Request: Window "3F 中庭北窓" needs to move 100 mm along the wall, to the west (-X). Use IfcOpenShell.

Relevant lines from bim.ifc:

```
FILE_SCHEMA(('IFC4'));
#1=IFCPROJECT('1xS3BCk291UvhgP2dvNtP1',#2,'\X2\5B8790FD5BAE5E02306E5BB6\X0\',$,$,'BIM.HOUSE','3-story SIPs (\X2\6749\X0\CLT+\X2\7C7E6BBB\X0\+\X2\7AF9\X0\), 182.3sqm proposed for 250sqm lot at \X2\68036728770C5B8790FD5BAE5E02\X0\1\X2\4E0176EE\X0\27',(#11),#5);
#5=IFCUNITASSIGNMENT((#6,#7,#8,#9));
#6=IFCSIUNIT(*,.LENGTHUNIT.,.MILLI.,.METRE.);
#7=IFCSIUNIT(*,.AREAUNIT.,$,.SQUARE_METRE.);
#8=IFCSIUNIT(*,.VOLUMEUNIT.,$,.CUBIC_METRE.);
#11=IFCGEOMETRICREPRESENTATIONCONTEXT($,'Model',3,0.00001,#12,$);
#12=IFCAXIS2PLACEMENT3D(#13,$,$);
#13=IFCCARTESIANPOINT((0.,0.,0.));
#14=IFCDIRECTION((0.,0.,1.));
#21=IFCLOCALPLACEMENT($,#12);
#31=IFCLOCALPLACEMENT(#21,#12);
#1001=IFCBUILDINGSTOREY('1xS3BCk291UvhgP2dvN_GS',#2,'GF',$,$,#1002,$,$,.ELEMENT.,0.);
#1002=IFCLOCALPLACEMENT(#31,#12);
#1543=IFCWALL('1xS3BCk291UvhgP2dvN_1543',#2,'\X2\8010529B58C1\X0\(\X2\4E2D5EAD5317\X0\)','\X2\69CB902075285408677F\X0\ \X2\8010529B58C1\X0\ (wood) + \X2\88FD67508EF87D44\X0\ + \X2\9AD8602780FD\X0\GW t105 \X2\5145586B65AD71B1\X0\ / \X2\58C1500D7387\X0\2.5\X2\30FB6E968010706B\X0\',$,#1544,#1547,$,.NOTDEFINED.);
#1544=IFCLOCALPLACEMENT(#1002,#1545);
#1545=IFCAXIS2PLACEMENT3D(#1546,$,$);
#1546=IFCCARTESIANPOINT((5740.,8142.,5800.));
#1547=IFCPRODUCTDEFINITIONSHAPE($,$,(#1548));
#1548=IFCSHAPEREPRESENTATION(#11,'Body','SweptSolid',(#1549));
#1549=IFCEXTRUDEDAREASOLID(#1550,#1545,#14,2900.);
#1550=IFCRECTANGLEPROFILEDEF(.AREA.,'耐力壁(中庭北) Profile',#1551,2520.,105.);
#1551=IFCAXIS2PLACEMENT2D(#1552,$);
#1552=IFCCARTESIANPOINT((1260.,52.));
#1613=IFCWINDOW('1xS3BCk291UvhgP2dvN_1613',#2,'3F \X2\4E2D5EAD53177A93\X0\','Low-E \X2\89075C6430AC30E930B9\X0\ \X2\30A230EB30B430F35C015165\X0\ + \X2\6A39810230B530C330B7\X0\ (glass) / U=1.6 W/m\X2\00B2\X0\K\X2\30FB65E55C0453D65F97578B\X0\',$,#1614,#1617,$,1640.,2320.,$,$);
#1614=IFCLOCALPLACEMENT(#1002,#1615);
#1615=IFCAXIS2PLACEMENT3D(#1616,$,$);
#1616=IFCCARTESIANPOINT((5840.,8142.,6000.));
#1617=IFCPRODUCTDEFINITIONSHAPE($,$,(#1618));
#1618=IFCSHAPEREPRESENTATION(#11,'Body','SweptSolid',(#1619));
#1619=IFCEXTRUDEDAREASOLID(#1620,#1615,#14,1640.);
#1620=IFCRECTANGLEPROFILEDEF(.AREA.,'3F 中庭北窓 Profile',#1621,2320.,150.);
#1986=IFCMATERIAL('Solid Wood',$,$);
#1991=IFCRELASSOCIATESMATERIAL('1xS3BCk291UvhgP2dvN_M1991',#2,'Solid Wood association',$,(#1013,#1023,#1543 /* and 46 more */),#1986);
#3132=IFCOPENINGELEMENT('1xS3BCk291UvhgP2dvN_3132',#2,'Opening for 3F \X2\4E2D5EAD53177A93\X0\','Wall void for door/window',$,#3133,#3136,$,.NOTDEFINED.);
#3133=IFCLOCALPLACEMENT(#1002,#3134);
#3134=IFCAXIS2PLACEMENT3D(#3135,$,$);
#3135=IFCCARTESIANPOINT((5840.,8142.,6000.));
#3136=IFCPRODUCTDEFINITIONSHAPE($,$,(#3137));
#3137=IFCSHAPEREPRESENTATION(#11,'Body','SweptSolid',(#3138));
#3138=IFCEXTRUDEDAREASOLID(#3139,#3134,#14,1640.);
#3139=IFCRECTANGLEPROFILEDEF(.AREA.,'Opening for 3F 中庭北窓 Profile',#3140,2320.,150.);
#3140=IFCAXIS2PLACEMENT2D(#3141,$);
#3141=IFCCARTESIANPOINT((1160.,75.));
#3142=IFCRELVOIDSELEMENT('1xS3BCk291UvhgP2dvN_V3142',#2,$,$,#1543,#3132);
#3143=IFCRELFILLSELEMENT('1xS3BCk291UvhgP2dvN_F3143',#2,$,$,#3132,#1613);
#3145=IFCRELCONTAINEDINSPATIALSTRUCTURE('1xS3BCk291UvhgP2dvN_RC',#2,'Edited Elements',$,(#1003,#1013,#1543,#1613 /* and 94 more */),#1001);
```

```python
import ifcopenshell
import ifcopenshell.api.geometry
import ifcopenshell.util.placement

model = ifcopenshell.open("bim.ifc")

window = model.by_id(1613)
opening = window.FillsVoids[0].RelatingOpeningElement
wall = opening.VoidsElements[0].RelatingBuildingElement

wall_matrix = ifcopenshell.util.placement.get_local_placement(wall.ObjectPlacement)
shift = wall_matrix[:3, 0] * -100.0
before = ifcopenshell.util.placement.get_local_placement(window.ObjectPlacement)[:3, 3].copy()

# The window is not placed relative to its opening, so move both.
for product in (opening, window):
    matrix = ifcopenshell.util.placement.get_local_placement(product.ObjectPlacement)
    matrix[:3, 3] += shift
    ifcopenshell.api.geometry.edit_object_placement(model, product=product, matrix=matrix, is_si=False)

after = ifcopenshell.util.placement.get_local_placement(window.ObjectPlacement)[:3, 3]
print("window moved by", (after - before).round(3) + 0.0)

model.write("bim_updated.ifc")
```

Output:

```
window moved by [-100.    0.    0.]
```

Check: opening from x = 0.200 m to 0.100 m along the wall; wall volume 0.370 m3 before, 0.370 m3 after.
